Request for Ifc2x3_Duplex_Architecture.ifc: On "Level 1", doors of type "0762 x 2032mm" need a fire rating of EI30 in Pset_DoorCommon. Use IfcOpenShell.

First a look at what the model holds.

```python
import ifcopenshell
import ifcopenshell.util.element

model = ifcopenshell.open("Ifc2x3_Duplex_Architecture.ifc")
print(model.schema)
storey = next(s for s in model.by_type("IfcBuildingStorey") if s.Name == "Level 1")
doors = [e for e in ifcopenshell.util.element.get_decomposition(storey) if e.is_a("IfcDoor")]
seen = {}
for e in doors:
    element_type = ifcopenshell.util.element.get_type(e)
    key = (element_type.Name if element_type != e and element_type else None, ifcopenshell.util.element.get_pset(e, "Pset_DoorCommon", "FireRating"))
    seen[key] = seen.get(key, 0) + 1
for (name, value), count in sorted(seen.items(), key=str):
    print(count, "x", name, "|", value)
```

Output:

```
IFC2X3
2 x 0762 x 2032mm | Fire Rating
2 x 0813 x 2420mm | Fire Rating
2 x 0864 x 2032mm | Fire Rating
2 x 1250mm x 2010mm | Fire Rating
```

```python
import ifcopenshell
import ifcopenshell.api.pset
import ifcopenshell.util.element

model = ifcopenshell.open("Ifc2x3_Duplex_Architecture.ifc")

storey = next(s for s in model.by_type("IfcBuildingStorey") if s.Name == "Level 1")
doors = [e for e in ifcopenshell.util.element.get_decomposition(storey) if e.is_a("IfcDoor")]

count = 0
for e in doors:
    element_type = ifcopenshell.util.element.get_type(e)
    if element_type in (None, e) or element_type.Name != "0762 x 2032mm":
        continue
    # add_pset returns the element's existing set when there is one.
    pset = ifcopenshell.api.pset.add_pset(model, product=e, name="Pset_DoorCommon")
    ifcopenshell.api.pset.edit_pset(model, pset=pset, properties={"FireRating": "EI30"})
    count += 1

print(count, "doors updated")

model.write("Ifc2x3_Duplex_Architecture_v2.ifc")
```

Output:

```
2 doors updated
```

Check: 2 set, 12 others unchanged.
